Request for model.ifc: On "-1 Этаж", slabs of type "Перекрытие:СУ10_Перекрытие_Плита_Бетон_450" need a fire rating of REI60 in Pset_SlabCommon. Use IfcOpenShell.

First a look at what the model holds.

```python
import ifcopenshell
import ifcopenshell.util.element

model = ifcopenshell.open("model.ifc")
print(model.schema)
storey = next(s for s in model.by_type("IfcBuildingStorey") if s.Name == "-1 Этаж")
slabs = [e for e in ifcopenshell.util.element.get_decomposition(storey) if e.is_a("IfcSlab")]
seen = {}
for e in slabs:
    element_type = ifcopenshell.util.element.get_type(e)
    key = (element_type.Name if element_type != e and element_type else None, ifcopenshell.util.element.get_pset(e, "Pset_SlabCommon", "FireRating"))
    seen[key] = seen.get(key, 0) + 1
for (name, value), count in sorted(seen.items(), key=str):
    print(count, "x", name, "|", value)
```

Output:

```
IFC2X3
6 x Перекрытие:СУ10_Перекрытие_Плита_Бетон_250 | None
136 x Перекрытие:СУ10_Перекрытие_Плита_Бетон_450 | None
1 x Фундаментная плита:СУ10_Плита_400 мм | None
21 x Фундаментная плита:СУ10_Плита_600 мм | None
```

```python
import ifcopenshell
import ifcopenshell.api.pset
import ifcopenshell.util.element

model = ifcopenshell.open("model.ifc")

storey = next(s for s in model.by_type("IfcBuildingStorey") if s.Name == "-1 Этаж")
slabs = [e for e in ifcopenshell.util.element.get_decomposition(storey) if e.is_a("IfcSlab")]

count = 0
for e in slabs:
    element_type = ifcopenshell.util.element.get_type(e)
    if element_type in (None, e) or element_type.Name != "Перекрытие:СУ10_Перекрытие_Плита_Бетон_450":
        continue
    # add_pset returns the element's existing set when there is one.
    pset = ifcopenshell.api.pset.add_pset(model, product=e, name="Pset_SlabCommon")
    ifcopenshell.api.pset.edit_pset(model, pset=pset, properties={"FireRating": "REI60"})
    count += 1

print(count, "slabs updated")

model.write("model-out.ifc")
```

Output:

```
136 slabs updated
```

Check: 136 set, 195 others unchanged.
